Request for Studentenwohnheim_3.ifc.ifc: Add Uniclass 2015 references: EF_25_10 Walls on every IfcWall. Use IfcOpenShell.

First a look at what the model holds.

```python
import ifcopenshell

model = ifcopenshell.open("Studentenwohnheim_3.ifc.ifc")
print(model.schema)
print("classifications:", [c.Name for c in model.by_type("IfcClassification")])
for ifc_class in ("IfcDoor", "IfcRoof", "IfcStair", "IfcWall", "IfcWindow"):
    print(ifc_class, len(model.by_type(ifc_class)))
```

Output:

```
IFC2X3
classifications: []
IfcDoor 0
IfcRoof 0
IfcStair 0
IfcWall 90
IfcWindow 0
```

```python
import ifcopenshell
import ifcopenshell.api.classification

model = ifcopenshell.open("Studentenwohnheim_3.ifc.ifc")

# IFC2X3 requires Source and Edition and has no link from the project to the system.
system = model.create_entity("IfcClassification", Source="NBS", Edition="2015", Name="Uniclass 2015")

codes = {
    "IfcWall": ("EF_25_10", "Walls"),
}
for ifc_class, (code, name) in codes.items():
    products = model.by_type(ifc_class)
    ifcopenshell.api.classification.add_reference(
        model, products=products, classification=system, identification=code, name=name
    )
    print(code, len(products))

model.write("Studentenwohnheim_3.ifc_rev.ifc")
```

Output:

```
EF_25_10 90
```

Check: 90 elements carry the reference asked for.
